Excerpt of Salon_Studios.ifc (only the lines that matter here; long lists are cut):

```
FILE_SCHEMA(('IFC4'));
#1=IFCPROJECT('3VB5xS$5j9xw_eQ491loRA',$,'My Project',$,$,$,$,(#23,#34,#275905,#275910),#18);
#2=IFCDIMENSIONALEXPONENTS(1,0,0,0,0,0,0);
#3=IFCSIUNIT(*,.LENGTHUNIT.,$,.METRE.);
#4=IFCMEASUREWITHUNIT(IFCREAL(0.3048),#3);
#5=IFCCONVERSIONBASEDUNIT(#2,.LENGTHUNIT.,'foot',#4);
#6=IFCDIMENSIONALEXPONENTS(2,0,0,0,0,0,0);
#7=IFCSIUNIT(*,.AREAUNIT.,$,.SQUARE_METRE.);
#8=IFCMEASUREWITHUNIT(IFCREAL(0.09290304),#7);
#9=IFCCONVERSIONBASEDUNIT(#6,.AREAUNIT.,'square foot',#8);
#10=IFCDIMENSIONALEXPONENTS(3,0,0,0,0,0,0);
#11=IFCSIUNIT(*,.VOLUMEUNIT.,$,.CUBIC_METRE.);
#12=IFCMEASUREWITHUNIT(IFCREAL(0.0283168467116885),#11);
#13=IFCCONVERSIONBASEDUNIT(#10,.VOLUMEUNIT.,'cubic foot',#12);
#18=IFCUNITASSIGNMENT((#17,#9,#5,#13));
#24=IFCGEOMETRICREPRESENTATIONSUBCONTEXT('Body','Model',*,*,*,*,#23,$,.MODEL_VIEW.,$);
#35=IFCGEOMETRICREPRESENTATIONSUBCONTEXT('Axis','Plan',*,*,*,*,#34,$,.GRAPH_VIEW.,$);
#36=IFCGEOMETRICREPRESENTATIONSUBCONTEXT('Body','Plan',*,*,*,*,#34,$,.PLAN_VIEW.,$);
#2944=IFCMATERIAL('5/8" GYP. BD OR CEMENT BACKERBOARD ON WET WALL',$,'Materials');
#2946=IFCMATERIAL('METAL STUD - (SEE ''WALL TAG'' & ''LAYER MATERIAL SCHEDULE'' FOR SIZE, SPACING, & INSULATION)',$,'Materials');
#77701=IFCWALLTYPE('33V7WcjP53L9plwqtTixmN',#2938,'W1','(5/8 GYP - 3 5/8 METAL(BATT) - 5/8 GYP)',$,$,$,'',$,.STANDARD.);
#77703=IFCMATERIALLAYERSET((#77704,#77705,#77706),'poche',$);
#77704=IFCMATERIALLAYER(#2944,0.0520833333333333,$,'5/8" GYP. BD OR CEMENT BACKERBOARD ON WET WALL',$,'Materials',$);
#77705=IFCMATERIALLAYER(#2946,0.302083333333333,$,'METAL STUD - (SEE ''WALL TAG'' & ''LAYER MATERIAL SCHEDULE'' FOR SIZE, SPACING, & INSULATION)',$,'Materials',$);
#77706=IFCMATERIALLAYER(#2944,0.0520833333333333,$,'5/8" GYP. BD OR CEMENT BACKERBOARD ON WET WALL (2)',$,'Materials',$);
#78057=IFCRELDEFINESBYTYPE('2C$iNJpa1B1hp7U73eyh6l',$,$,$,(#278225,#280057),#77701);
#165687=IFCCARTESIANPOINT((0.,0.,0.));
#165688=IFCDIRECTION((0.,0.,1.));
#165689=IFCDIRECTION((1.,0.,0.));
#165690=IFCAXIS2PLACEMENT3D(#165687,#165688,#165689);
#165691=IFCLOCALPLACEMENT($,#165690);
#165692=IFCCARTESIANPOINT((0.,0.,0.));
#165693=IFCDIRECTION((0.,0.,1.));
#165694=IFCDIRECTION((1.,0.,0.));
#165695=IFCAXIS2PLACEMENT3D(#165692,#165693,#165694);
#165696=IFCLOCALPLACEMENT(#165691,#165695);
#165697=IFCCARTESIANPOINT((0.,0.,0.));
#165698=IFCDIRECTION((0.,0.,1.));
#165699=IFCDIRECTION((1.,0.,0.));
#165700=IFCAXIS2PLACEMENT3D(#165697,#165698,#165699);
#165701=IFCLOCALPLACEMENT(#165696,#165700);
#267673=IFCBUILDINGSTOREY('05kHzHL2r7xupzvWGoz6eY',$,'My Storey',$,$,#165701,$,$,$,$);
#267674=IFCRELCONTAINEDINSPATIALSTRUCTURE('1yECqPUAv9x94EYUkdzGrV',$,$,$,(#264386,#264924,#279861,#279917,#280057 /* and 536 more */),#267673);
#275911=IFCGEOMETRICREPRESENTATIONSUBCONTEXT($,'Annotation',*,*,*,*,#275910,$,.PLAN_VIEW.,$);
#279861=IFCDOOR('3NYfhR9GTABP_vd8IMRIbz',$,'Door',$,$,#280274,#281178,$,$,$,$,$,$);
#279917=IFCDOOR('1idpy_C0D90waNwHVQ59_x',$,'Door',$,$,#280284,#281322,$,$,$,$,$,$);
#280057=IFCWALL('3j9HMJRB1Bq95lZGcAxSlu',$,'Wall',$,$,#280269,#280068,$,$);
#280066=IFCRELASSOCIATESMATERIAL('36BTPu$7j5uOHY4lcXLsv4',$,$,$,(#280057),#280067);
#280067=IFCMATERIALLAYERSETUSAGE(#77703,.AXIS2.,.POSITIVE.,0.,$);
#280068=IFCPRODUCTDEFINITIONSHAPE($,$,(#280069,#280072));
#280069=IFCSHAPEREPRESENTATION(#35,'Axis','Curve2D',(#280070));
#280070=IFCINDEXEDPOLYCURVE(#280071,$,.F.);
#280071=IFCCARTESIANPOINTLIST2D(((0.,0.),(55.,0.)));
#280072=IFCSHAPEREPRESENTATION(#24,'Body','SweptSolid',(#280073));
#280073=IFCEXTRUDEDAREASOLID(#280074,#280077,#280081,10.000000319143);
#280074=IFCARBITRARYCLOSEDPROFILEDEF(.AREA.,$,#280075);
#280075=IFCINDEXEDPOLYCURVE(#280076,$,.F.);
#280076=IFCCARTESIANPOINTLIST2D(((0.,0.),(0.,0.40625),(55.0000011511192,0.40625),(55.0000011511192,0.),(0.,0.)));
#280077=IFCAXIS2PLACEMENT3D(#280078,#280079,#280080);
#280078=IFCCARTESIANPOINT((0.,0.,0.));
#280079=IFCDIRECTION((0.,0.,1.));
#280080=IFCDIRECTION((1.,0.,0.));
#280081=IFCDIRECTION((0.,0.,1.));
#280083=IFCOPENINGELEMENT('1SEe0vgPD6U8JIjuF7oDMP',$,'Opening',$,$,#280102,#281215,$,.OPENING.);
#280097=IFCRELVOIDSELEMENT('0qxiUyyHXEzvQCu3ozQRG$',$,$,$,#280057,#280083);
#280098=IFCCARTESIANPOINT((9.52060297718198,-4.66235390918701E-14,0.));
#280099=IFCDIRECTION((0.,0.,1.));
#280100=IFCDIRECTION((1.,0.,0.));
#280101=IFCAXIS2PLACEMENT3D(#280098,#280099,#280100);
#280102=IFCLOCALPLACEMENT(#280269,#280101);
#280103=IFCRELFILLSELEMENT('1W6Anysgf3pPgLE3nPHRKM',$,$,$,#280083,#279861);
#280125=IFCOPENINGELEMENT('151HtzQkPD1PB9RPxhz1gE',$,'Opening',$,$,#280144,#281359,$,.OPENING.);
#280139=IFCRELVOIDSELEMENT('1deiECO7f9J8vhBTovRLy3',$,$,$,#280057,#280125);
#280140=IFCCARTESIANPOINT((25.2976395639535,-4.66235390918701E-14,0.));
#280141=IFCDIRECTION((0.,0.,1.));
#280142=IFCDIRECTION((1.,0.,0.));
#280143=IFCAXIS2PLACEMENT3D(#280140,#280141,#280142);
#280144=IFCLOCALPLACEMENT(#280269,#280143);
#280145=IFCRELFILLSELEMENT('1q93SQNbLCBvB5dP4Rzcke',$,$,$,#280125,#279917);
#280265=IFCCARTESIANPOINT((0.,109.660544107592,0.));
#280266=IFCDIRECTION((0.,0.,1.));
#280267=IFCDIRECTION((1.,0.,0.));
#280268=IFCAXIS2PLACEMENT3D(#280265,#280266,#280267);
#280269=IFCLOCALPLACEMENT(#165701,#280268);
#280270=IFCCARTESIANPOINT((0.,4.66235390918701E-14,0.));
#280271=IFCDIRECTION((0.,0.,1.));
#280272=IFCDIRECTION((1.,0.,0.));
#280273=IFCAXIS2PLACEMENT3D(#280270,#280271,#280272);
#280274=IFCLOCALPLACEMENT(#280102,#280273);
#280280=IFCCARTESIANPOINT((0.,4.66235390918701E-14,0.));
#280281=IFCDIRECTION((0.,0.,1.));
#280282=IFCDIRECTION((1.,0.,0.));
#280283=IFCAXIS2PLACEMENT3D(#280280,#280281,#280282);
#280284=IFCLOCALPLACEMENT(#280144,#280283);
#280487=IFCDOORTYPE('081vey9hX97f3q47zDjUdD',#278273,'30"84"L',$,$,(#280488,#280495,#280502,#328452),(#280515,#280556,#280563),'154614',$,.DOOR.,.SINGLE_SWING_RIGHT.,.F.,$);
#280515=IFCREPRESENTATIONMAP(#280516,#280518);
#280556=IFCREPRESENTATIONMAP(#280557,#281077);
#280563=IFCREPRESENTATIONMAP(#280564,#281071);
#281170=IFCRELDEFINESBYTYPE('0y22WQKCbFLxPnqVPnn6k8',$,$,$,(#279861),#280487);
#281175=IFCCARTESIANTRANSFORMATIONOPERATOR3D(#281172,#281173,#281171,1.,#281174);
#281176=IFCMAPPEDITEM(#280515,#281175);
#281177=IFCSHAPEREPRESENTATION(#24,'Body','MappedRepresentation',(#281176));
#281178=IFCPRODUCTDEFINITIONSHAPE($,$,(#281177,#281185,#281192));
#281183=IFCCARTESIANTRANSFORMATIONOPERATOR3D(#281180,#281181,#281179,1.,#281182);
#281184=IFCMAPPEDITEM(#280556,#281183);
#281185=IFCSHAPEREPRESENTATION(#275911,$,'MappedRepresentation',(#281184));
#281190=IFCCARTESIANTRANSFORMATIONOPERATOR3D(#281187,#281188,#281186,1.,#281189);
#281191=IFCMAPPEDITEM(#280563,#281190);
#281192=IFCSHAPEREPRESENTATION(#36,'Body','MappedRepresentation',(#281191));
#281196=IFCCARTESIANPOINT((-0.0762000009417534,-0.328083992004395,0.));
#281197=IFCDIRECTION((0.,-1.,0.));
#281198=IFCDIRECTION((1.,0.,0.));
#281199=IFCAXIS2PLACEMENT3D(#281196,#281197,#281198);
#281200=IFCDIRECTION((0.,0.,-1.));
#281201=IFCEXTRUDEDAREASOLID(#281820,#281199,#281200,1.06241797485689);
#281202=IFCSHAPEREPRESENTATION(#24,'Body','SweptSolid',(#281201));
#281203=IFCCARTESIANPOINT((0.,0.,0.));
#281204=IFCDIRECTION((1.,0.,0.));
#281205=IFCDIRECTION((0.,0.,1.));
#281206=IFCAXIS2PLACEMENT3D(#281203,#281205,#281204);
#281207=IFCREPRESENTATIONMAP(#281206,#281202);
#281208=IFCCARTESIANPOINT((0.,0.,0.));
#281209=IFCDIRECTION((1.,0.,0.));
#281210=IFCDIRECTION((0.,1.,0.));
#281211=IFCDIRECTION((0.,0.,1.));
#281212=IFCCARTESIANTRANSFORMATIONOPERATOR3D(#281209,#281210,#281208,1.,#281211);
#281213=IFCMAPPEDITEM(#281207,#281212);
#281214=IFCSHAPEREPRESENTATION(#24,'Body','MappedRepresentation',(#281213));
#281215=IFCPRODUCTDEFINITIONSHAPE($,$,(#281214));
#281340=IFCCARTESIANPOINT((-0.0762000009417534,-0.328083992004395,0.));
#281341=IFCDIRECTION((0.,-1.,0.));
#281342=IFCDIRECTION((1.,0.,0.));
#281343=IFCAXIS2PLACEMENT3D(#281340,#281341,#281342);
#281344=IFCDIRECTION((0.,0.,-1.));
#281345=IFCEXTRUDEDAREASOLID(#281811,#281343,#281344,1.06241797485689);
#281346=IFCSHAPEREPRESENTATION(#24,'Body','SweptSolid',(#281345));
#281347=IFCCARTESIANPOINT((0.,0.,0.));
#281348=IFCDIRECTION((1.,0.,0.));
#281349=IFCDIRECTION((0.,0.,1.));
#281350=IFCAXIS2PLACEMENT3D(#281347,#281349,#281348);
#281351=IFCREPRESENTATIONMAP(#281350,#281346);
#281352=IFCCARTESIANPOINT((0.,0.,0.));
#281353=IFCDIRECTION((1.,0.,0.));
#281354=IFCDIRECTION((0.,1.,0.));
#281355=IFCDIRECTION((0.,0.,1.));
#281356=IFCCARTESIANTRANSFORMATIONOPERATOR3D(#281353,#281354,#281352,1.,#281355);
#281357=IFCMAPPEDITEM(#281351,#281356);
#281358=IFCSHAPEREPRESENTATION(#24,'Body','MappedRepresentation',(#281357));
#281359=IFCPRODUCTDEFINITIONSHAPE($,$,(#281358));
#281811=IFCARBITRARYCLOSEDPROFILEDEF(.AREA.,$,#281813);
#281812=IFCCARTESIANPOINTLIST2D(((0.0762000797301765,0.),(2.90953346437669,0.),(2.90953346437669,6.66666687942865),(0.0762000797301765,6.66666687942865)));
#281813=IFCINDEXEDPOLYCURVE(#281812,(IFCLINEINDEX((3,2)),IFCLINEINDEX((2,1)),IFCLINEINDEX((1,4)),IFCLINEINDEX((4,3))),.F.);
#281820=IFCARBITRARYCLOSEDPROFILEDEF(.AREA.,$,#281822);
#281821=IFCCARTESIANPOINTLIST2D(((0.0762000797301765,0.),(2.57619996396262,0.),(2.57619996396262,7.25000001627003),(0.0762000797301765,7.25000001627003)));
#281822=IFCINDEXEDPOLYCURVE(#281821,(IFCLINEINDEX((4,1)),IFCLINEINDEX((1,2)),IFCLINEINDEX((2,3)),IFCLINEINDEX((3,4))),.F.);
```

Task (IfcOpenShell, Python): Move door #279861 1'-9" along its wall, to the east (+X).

```python
import ifcopenshell
import ifcopenshell.api.geometry
import ifcopenshell.util.placement
import ifcopenshell.util.unit

model = ifcopenshell.open("Salon_Studios.ifc")
unit_scale = ifcopenshell.util.unit.calculate_unit_scale(model)

door = model.by_guid("3NYfhR9GTABP_vd8IMRIbz")
opening = door.FillsVoids[0].RelatingOpeningElement
wall = opening.VoidsElements[0].RelatingBuildingElement

wall_matrix = ifcopenshell.util.placement.get_local_placement(wall.ObjectPlacement)
shift = wall_matrix[:3, 0] * 21 * 0.0254 / unit_scale
before = ifcopenshell.util.placement.get_local_placement(door.ObjectPlacement)[:3, 3].copy()

# The door is placed relative to its opening, so it follows when the opening moves.
matrix = ifcopenshell.util.placement.get_local_placement(opening.ObjectPlacement)
matrix[:3, 3] += shift
ifcopenshell.api.geometry.edit_object_placement(
    model, product=opening, matrix=matrix, is_si=False, should_transform_children=True
)

after = ifcopenshell.util.placement.get_local_placement(door.ObjectPlacement)[:3, 3]
print("door moved by", (after - before).round(3) + 0.0)

model.write("Salon_Studios_rev.ifc")
```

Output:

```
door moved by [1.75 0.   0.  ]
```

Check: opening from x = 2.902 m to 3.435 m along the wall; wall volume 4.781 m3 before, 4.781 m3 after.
